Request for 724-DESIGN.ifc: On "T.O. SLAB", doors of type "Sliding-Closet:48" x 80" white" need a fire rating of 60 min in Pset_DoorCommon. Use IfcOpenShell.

First a look at what the model holds.

```python
import ifcopenshell
import ifcopenshell.util.element

model = ifcopenshell.open("724-DESIGN.ifc")
print(model.schema)
storey = next(s for s in model.by_type("IfcBuildingStorey") if s.Name == "T.O. SLAB")
doors = [e for e in ifcopenshell.util.element.get_decomposition(storey) if e.is_a("IfcDoor")]
seen = {}
for e in doors:
    element_type = ifcopenshell.util.element.get_type(e)
    key = (element_type.Name if element_type != e and element_type else None, ifcopenshell.util.element.get_pset(e, "Pset_DoorCommon", "FireRating"))
    seen[key] = seen.get(key, 0) + 1
for (name, value), count in sorted(seen.items(), key=str):
    print(count, "x", name, "|", value)
```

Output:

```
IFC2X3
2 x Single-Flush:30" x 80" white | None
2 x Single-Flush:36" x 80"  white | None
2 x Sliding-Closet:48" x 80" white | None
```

```python
import ifcopenshell
import ifcopenshell.api.pset
import ifcopenshell.util.element

model = ifcopenshell.open("724-DESIGN.ifc")

storey = next(s for s in model.by_type("IfcBuildingStorey") if s.Name == "T.O. SLAB")
doors = [e for e in ifcopenshell.util.element.get_decomposition(storey) if e.is_a("IfcDoor")]

count = 0
for e in doors:
    element_type = ifcopenshell.util.element.get_type(e)
    if element_type in (None, e) or element_type.Name != 'Sliding-Closet:48" x 80" white':
        continue
    # add_pset returns the element's existing set when there is one.
    pset = ifcopenshell.api.pset.add_pset(model, product=e, name="Pset_DoorCommon")
    ifcopenshell.api.pset.edit_pset(model, pset=pset, properties={"FireRating": "60 min"})
    count += 1

print(count, "doors updated")

model.write("724-DESIGN-out.ifc")
```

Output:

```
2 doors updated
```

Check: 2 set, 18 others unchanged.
